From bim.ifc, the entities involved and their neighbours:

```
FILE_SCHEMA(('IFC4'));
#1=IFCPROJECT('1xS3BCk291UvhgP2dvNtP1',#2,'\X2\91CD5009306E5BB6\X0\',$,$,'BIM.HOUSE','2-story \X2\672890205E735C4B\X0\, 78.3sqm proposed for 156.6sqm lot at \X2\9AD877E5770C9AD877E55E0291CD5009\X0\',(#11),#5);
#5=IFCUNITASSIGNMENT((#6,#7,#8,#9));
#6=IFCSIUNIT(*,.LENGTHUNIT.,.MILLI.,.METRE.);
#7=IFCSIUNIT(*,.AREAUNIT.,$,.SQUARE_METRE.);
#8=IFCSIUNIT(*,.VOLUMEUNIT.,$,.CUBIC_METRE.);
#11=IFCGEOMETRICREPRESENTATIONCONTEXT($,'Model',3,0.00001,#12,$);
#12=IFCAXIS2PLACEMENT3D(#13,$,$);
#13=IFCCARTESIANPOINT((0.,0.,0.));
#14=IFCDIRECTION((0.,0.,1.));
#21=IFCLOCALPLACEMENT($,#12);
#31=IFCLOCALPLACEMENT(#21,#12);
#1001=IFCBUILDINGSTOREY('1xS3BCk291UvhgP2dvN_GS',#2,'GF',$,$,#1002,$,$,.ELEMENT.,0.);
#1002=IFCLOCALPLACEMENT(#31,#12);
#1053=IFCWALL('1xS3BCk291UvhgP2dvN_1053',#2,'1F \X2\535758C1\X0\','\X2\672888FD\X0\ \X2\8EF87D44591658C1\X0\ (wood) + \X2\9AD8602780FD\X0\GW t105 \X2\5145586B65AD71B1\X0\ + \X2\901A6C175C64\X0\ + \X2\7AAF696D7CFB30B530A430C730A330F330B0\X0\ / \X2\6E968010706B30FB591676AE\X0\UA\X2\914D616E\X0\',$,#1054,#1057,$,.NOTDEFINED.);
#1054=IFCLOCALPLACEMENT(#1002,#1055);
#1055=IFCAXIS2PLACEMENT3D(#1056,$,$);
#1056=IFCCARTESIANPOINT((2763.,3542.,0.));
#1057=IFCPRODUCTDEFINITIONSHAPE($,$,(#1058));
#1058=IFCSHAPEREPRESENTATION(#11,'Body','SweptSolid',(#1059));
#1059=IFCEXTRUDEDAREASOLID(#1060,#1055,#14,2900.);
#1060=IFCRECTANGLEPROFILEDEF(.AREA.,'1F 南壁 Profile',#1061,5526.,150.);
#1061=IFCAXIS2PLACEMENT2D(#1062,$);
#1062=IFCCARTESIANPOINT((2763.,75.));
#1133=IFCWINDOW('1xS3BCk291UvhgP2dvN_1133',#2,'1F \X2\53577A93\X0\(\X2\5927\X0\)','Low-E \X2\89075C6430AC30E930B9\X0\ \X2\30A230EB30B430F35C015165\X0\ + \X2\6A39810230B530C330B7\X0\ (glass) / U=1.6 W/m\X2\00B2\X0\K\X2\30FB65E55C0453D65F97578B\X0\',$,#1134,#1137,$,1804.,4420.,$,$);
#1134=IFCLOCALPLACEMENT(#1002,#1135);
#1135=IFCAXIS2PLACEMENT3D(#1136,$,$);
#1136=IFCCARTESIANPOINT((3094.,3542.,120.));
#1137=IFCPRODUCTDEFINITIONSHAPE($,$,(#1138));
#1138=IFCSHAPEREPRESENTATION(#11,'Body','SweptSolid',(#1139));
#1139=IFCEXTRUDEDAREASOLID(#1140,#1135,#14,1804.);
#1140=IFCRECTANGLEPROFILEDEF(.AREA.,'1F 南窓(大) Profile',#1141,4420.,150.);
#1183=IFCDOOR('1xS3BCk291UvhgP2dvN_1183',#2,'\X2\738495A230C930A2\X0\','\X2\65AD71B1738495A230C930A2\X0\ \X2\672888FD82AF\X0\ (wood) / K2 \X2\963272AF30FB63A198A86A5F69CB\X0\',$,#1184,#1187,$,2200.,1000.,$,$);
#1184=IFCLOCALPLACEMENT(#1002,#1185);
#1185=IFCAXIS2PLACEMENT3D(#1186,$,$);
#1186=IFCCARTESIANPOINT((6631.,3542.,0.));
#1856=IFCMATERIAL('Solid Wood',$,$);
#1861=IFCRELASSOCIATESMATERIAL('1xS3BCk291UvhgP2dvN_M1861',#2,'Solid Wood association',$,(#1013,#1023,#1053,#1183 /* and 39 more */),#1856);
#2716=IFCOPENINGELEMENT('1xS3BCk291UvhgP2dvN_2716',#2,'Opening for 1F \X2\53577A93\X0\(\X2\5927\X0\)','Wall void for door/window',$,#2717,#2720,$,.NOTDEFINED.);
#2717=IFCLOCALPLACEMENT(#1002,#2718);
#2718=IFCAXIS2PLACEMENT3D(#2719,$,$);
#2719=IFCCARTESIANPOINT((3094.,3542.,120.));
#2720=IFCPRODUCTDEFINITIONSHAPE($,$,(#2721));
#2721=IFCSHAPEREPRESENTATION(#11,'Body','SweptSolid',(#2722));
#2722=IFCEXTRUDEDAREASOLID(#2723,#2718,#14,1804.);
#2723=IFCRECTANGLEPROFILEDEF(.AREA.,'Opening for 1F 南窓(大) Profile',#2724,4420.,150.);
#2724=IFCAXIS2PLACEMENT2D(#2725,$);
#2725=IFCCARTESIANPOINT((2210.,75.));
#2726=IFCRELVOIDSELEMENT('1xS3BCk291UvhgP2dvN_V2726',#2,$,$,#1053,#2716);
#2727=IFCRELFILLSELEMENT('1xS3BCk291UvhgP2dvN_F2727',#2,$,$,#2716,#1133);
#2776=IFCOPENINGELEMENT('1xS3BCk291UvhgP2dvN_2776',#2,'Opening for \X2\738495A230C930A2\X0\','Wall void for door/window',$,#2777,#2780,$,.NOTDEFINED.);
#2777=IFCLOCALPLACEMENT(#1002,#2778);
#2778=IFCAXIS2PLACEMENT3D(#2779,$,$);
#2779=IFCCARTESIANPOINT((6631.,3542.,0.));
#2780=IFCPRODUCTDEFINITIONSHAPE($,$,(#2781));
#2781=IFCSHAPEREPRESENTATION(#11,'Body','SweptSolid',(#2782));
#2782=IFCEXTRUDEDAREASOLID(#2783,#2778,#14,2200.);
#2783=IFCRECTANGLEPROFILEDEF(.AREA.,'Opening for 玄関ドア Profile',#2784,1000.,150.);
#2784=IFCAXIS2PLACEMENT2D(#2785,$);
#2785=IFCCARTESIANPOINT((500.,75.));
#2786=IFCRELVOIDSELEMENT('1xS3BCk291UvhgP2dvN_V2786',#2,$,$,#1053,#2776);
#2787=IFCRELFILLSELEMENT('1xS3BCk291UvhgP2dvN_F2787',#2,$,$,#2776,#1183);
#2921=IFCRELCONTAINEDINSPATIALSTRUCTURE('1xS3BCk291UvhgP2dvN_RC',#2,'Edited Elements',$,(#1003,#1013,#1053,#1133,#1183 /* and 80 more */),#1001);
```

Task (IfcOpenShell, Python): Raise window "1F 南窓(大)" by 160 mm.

```python
import numpy as np
import ifcopenshell
import ifcopenshell.api.geometry
import ifcopenshell.util.placement
import ifcopenshell.util.unit

model = ifcopenshell.open("bim.ifc")
unit_scale = ifcopenshell.util.unit.calculate_unit_scale(model)

window = model.by_guid("1xS3BCk291UvhgP2dvN_1133")
opening = window.FillsVoids[0].RelatingOpeningElement
dz = 160.0

shift = np.array([0.0, 0.0, dz])
# The window is not placed relative to its opening, so move both.
for product in (opening, window):
    matrix = ifcopenshell.util.placement.get_local_placement(product.ObjectPlacement)
    matrix[:3, 3] += shift
    ifcopenshell.api.geometry.edit_object_placement(model, product=product, matrix=matrix, is_si=False)

print(f"moved by {dz * unit_scale:+.3f} m")

model.write("bim_updated.ifc")
```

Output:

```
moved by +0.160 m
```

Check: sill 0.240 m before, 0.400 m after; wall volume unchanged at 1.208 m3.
